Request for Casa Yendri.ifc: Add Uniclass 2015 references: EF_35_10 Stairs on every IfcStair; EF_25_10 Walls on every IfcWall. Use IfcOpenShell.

First a look at what the model holds.

```python
import ifcopenshell

model = ifcopenshell.open("Casa Yendri.ifc")
print(model.schema)
print("classifications:", [c.Name for c in model.by_type("IfcClassification")])
for ifc_class in ("IfcDoor", "IfcRoof", "IfcStair", "IfcWall", "IfcWindow"):
    print(ifc_class, len(model.by_type(ifc_class)))
```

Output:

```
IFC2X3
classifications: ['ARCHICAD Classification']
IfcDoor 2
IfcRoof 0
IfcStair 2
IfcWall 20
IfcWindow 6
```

```python
import ifcopenshell
import ifcopenshell.api.classification

model = ifcopenshell.open("Casa Yendri.ifc")

# IFC2X3 requires Source and Edition and has no link from the project to the system.
system = model.create_entity("IfcClassification", Source="NBS", Edition="2015", Name="Uniclass 2015")

codes = {
    "IfcStair": ("EF_35_10", "Stairs"),
    "IfcWall": ("EF_25_10", "Walls"),
}
for ifc_class, (code, name) in codes.items():
    products = model.by_type(ifc_class)
    ifcopenshell.api.classification.add_reference(
        model, products=products, classification=system, identification=code, name=name
    )
    print(code, len(products))

model.write("Casa Yendri_v2.ifc")
```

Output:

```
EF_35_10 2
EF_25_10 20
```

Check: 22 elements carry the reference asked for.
